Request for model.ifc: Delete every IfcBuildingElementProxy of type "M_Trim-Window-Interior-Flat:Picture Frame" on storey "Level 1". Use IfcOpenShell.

First a look at what the model holds.

```python
import ifcopenshell
import ifcopenshell.util.element

model = ifcopenshell.open("model.ifc")
print(model.schema)
storey = next(s for s in model.by_type("IfcBuildingStorey") if s.Name == "Level 1")
proxies = [e for e in ifcopenshell.util.element.get_decomposition(storey) if e.is_a("IfcBuildingElementProxy")]
seen = {}
for e in proxies:
    element_type = ifcopenshell.util.element.get_type(e)
    name = element_type.Name if element_type not in (None, e) else None
    seen[name] = seen.get(name, 0) + 1
for name, count in sorted(seen.items(), key=str):
    print(count, "x", name)
```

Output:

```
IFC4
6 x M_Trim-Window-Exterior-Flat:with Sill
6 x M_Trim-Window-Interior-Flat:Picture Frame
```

```python
import ifcopenshell
import ifcopenshell.api.root
import ifcopenshell.util.element

model = ifcopenshell.open("model.ifc")

storey = next(s for s in model.by_type("IfcBuildingStorey") if s.Name == "Level 1")
proxies = [e for e in ifcopenshell.util.element.get_decomposition(storey) if e.is_a("IfcBuildingElementProxy")]
targets = [e for e in proxies if (t := ifcopenshell.util.element.get_type(e)) not in (None, e) and t.Name == "M_Trim-Window-Interior-Flat:Picture Frame"]

for e in targets:
    ifcopenshell.api.root.remove_product(model, product=e)
print(len(targets), "removed")

model.write("model_updated.ifc")
```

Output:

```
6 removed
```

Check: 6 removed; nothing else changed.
